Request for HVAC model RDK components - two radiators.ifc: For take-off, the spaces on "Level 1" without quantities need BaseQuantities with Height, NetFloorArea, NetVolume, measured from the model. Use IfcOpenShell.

First a look at what the model holds.

```python
import ifcopenshell
import ifcopenshell.util.element
import ifcopenshell.util.unit

model = ifcopenshell.open("HVAC model RDK components - two radiators.ifc")
print(model.schema)
for unit_type in ("LENGTHUNIT", "AREAUNIT", "VOLUMEUNIT"):
    print(unit_type, ifcopenshell.util.unit.calculate_unit_scale(model, unit_type))
storey = next(s for s in model.by_type("IfcBuildingStorey") if s.Name == "Level 1")
spaces = [e for e in ifcopenshell.util.element.get_decomposition(storey) if e.is_a("IfcSpace")]
for e in sorted(spaces, key=lambda e: e.id()):
    print(e.id(), e.is_a(), e.Name, list(ifcopenshell.util.element.get_psets(e, qtos_only=True)), sep=" | ")
```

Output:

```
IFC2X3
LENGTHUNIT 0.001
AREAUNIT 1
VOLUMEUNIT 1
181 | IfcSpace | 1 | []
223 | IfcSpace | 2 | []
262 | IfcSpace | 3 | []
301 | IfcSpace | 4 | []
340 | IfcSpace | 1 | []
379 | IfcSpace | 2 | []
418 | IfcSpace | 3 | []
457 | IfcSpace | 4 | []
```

```python
import ifcopenshell
import ifcopenshell.api.pset
import ifcopenshell.geom
import ifcopenshell.util.element
import ifcopenshell.util.shape
import ifcopenshell.util.unit

model = ifcopenshell.open("HVAC model RDK components - two radiators.ifc")
unit_scale = ifcopenshell.util.unit.calculate_unit_scale(model)
area_scale = ifcopenshell.util.unit.calculate_unit_scale(model, "AREAUNIT")
volume_scale = ifcopenshell.util.unit.calculate_unit_scale(model, "VOLUMEUNIT")
settings = ifcopenshell.geom.settings()

storey = next(s for s in model.by_type("IfcBuildingStorey") if s.Name == "Level 1")
spaces = [e for e in ifcopenshell.util.element.get_decomposition(storey) if e.is_a("IfcSpace")]

for e in sorted(spaces, key=lambda e: e.id()):
    if ifcopenshell.util.element.get_psets(e, qtos_only=True, should_inherit=False):
        continue
    # Geometry comes back in metres, in the element's own axes.
    shape = ifcopenshell.geom.create_shape(settings, e)
    values = {
        "Height": ifcopenshell.util.shape.get_z(shape.geometry) / unit_scale,
        "NetFloorArea": ifcopenshell.util.shape.get_footprint_area(shape.geometry) / area_scale,
        "NetVolume": ifcopenshell.util.shape.get_volume(shape.geometry) / volume_scale,
    }
    qto = ifcopenshell.api.pset.add_qto(model, product=e, name="BaseQuantities")
    ifcopenshell.api.pset.edit_qto(model, qto=qto, properties=values)
    print(e.id(), {k: round(v, 3) for k, v in values.items()})

model.write("HVAC model RDK components - two radiators_v2.ifc")
```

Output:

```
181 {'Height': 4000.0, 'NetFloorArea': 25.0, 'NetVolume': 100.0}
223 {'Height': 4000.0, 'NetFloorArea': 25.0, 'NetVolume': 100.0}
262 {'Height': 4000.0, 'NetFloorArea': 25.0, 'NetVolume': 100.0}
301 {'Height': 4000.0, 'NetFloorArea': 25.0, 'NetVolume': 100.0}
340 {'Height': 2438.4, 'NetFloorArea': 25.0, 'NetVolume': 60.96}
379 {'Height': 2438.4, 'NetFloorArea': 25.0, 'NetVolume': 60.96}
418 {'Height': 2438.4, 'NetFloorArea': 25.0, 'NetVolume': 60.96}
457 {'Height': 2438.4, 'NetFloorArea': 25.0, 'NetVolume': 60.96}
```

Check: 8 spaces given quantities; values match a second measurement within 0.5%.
